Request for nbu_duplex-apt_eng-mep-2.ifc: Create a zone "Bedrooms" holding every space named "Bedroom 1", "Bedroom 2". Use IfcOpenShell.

First a look at what the model holds.

```python
import ifcopenshell

model = ifcopenshell.open("nbu_duplex-apt_eng-mep-2.ifc")
print(model.schema)
seen = {}
for space in model.by_type("IfcSpace"):
    seen[space.LongName] = seen.get(space.LongName, 0) + 1
for name, count in sorted(seen.items(), key=str):
    print(count, "x", name)
print("zones:", [z.Name for z in model.by_type("IfcZone")][:20])
```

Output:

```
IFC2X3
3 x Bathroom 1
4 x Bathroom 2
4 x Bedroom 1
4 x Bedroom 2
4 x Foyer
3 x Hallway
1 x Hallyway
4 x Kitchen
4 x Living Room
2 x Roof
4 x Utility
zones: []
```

```python
import ifcopenshell
import ifcopenshell.api.group
import ifcopenshell.api.root

model = ifcopenshell.open("nbu_duplex-apt_eng-mep-2.ifc")

names = {"Bedroom 1", "Bedroom 2"}
spaces = [s for s in model.by_type("IfcSpace") if s.LongName in names]

zone = ifcopenshell.api.root.create_entity(model, ifc_class="IfcZone", name="Bedrooms")
ifcopenshell.api.group.assign_group(model, products=spaces, group=zone)
print(len(spaces), "spaces in", zone.Name)

model.write("nbu_duplex-apt_eng-mep-2_v2.ifc")
```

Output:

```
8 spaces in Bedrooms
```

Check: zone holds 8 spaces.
